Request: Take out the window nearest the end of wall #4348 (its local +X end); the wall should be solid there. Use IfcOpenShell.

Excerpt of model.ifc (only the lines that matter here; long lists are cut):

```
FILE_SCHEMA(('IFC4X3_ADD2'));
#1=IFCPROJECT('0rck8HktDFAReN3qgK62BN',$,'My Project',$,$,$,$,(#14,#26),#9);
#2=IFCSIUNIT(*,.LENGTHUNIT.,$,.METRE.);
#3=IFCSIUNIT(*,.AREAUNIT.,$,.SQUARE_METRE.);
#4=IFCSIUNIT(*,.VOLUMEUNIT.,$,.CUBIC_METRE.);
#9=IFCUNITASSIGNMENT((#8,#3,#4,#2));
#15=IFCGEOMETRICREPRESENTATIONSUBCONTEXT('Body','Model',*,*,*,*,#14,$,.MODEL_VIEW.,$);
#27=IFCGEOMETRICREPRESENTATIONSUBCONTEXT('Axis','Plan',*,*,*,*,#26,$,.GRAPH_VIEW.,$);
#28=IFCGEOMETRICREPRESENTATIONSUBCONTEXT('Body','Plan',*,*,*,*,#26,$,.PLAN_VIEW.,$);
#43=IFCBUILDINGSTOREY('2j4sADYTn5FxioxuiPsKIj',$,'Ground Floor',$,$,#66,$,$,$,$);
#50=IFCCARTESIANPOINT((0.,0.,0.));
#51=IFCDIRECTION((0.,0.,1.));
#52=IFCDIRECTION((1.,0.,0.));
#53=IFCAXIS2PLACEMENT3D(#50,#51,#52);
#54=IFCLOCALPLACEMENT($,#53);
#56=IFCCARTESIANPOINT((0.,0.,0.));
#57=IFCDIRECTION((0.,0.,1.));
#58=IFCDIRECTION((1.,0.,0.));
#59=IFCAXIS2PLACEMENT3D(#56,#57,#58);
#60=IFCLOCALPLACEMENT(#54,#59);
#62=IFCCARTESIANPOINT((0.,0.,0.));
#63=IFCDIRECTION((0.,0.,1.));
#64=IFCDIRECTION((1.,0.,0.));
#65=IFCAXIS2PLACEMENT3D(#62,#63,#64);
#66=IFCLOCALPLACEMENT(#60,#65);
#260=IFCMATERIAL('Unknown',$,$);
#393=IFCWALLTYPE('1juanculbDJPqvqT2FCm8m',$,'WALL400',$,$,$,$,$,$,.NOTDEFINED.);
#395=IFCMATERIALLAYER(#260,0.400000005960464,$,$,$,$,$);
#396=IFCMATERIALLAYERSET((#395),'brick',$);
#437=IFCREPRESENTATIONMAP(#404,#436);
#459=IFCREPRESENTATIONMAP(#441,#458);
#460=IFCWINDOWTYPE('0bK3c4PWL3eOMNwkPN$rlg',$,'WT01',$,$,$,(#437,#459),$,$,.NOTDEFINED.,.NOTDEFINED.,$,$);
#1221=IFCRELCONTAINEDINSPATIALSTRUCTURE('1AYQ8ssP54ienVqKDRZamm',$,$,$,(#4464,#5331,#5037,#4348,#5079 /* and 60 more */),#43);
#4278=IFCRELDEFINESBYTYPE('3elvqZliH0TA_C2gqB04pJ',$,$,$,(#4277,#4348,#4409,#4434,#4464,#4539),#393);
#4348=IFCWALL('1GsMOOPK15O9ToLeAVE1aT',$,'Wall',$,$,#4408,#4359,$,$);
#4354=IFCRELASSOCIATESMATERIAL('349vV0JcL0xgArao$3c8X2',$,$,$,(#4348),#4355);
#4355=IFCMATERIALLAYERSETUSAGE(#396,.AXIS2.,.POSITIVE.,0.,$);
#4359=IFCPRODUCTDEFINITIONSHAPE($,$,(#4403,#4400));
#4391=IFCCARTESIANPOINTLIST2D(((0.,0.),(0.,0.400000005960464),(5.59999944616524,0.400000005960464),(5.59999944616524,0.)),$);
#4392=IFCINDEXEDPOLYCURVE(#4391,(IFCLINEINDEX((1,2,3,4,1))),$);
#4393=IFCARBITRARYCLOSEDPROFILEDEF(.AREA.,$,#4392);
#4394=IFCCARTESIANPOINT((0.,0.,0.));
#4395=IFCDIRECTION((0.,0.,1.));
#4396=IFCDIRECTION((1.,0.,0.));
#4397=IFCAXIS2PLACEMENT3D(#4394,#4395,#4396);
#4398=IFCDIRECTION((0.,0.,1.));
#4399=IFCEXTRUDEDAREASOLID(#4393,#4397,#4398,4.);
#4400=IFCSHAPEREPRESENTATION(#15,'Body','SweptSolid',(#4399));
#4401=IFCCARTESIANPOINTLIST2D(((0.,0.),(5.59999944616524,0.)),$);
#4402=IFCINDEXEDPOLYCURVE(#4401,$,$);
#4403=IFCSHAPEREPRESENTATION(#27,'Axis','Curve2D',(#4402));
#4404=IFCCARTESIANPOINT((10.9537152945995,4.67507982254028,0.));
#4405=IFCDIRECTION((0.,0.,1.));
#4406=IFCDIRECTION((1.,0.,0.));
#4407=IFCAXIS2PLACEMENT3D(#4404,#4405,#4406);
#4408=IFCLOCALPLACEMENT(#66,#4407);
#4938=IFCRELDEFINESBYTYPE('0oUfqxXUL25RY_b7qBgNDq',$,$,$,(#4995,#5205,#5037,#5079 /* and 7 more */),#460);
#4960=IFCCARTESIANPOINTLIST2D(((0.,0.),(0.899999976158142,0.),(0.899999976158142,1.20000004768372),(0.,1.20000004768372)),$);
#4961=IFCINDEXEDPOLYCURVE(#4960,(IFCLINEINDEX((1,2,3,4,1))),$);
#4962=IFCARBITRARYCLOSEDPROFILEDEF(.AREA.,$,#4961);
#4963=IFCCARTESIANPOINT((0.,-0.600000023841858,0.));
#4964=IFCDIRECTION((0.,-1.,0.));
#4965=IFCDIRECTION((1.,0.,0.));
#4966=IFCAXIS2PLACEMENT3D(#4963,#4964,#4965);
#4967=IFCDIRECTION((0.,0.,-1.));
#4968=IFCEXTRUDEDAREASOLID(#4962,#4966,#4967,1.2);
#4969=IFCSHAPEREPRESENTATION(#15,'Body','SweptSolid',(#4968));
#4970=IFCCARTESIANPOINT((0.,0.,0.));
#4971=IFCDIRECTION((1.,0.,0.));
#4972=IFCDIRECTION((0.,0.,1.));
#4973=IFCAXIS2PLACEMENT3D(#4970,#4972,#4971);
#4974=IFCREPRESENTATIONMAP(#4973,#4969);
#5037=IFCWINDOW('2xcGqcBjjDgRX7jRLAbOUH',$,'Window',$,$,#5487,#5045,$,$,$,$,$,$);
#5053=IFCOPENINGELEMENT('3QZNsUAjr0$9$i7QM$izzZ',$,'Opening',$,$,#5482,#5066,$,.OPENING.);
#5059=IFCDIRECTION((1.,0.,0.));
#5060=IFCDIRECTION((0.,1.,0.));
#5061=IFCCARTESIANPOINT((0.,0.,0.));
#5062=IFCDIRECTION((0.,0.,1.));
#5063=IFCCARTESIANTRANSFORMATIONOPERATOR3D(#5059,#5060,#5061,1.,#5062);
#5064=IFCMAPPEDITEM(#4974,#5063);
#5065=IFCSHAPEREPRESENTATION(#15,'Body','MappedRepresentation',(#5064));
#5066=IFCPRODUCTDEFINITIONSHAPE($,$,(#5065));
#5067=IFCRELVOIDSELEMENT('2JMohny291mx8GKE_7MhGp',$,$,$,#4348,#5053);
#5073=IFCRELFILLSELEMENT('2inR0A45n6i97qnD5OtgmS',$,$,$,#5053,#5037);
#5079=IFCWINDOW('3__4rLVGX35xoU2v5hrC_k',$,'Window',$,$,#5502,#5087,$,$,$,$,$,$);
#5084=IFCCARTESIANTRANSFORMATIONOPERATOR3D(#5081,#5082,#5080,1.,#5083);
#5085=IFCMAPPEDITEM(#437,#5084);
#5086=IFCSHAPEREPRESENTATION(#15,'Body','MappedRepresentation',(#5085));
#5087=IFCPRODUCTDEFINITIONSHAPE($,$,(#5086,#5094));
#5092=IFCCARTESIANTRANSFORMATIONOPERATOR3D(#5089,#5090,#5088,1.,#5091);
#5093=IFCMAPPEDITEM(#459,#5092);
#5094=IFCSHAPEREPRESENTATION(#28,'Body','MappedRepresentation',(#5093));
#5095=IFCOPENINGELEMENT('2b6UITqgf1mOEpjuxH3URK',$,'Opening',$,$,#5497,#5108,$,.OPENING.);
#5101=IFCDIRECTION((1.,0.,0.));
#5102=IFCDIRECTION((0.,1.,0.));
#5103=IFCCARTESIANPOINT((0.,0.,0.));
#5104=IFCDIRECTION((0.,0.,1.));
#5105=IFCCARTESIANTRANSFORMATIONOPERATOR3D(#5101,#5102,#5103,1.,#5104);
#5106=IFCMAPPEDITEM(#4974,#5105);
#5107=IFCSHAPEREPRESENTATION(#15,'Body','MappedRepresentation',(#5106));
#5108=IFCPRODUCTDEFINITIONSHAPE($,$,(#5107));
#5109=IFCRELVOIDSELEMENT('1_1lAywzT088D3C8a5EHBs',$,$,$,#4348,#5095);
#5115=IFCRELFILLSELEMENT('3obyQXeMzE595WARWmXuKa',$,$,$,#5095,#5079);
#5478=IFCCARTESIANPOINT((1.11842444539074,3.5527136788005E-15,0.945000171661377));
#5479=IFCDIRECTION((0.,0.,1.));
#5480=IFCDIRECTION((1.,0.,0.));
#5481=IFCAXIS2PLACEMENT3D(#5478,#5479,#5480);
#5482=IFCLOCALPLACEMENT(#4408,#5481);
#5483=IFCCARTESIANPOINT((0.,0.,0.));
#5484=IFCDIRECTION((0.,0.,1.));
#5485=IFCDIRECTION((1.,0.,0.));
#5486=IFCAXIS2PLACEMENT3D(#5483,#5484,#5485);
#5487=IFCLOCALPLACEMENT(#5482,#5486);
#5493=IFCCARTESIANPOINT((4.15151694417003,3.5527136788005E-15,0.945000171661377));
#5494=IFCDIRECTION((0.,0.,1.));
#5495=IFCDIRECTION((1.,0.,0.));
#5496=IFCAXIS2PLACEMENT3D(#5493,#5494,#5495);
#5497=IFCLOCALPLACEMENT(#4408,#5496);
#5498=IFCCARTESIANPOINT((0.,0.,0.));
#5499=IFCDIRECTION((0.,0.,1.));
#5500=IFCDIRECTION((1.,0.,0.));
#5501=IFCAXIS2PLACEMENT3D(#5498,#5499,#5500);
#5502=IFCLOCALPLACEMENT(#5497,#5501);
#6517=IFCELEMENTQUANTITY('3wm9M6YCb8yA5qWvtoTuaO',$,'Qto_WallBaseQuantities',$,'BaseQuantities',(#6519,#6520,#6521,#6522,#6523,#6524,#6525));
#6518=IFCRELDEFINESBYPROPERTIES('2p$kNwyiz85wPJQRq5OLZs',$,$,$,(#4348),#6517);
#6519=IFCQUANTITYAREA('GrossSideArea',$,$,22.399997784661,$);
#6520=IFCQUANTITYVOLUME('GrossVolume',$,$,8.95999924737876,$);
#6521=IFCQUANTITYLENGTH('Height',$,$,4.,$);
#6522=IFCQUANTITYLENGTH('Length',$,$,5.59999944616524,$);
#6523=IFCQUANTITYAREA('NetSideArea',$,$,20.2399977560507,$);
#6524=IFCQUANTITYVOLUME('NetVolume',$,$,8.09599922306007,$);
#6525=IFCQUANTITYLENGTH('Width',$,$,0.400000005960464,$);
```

```python
import ifcopenshell
import ifcopenshell.api.feature
import ifcopenshell.api.pset
import ifcopenshell.api.root
import ifcopenshell.geom
import ifcopenshell.util.element
import ifcopenshell.util.shape
import ifcopenshell.util.unit

model = ifcopenshell.open("model.ifc")
area_scale = ifcopenshell.util.unit.calculate_unit_scale(model, "AREAUNIT")
volume_scale = ifcopenshell.util.unit.calculate_unit_scale(model, "VOLUMEUNIT")
settings = ifcopenshell.geom.settings()


def volume(element):
    """Net volume in cubic metres, openings subtracted."""
    shape = ifcopenshell.geom.create_shape(settings, element)
    return ifcopenshell.util.shape.get_volume(shape.geometry)


window = model.by_guid("3__4rLVGX35xoU2v5hrC_k")
opening = window.FillsVoids[0].RelatingOpeningElement
wall = opening.VoidsElements[0].RelatingBuildingElement
before = volume(wall)

ifcopenshell.api.root.remove_product(model, product=window)
ifcopenshell.api.feature.remove_feature(model, feature=opening)

after = volume(wall)
thickness = 0.4  # wall thickness in metres

# Update the wall's stored quantities.
qto = model.by_id(ifcopenshell.util.element.get_pset(wall, "Qto_WallBaseQuantities", should_inherit=False)["id"])
ifcopenshell.api.pset.edit_qto(model, qto=qto, properties={
    "NetSideArea": after / thickness / area_scale,
    "NetVolume": after / volume_scale,
})

print(f"wall volume {before:.3f} -> {after:.3f} m3")

model.write("model_updated.ifc")
```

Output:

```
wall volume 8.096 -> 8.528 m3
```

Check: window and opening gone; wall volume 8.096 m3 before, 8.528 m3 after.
